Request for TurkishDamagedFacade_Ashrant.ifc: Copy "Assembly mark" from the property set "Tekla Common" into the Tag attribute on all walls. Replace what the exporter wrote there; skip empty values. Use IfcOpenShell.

First a look at what the model holds.

```python
import ifcopenshell
import ifcopenshell.util.element

model = ifcopenshell.open("TurkishDamagedFacade_Ashrant.ifc")
print(model.schema)
walls = model.by_type("IfcWall")
print(len(walls), "walls")
for e in walls[:8]:
    source = ifcopenshell.util.element.get_pset(e, "Tekla Common", "Assembly mark")
    target = e.Tag
    print(e.id(), repr(source), repr(target), sep=" | ")
```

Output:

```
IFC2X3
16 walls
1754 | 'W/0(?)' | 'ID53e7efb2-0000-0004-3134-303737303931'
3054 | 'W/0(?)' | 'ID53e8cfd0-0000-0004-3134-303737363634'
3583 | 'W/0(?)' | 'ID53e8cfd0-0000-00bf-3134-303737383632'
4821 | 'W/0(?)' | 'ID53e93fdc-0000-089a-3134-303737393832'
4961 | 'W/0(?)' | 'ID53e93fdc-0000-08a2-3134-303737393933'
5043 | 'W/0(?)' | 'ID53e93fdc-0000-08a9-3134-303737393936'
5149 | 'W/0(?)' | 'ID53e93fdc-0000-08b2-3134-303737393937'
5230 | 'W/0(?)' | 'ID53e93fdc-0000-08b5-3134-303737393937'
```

```python
import ifcopenshell
import ifcopenshell.util.element

model = ifcopenshell.open("TurkishDamagedFacade_Ashrant.ifc")

count = 0
for e in model.by_type("IfcWall"):
    value = ifcopenshell.util.element.get_pset(e, "Tekla Common", "Assembly mark")
    current = e.Tag
    if not value or not value.strip() or current == value:
        continue
    e.Tag = value
    count += 1

print(count, "walls updated")

model.write("TurkishDamagedFacade_Ashrant-out.ifc")
```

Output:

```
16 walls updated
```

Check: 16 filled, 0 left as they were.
